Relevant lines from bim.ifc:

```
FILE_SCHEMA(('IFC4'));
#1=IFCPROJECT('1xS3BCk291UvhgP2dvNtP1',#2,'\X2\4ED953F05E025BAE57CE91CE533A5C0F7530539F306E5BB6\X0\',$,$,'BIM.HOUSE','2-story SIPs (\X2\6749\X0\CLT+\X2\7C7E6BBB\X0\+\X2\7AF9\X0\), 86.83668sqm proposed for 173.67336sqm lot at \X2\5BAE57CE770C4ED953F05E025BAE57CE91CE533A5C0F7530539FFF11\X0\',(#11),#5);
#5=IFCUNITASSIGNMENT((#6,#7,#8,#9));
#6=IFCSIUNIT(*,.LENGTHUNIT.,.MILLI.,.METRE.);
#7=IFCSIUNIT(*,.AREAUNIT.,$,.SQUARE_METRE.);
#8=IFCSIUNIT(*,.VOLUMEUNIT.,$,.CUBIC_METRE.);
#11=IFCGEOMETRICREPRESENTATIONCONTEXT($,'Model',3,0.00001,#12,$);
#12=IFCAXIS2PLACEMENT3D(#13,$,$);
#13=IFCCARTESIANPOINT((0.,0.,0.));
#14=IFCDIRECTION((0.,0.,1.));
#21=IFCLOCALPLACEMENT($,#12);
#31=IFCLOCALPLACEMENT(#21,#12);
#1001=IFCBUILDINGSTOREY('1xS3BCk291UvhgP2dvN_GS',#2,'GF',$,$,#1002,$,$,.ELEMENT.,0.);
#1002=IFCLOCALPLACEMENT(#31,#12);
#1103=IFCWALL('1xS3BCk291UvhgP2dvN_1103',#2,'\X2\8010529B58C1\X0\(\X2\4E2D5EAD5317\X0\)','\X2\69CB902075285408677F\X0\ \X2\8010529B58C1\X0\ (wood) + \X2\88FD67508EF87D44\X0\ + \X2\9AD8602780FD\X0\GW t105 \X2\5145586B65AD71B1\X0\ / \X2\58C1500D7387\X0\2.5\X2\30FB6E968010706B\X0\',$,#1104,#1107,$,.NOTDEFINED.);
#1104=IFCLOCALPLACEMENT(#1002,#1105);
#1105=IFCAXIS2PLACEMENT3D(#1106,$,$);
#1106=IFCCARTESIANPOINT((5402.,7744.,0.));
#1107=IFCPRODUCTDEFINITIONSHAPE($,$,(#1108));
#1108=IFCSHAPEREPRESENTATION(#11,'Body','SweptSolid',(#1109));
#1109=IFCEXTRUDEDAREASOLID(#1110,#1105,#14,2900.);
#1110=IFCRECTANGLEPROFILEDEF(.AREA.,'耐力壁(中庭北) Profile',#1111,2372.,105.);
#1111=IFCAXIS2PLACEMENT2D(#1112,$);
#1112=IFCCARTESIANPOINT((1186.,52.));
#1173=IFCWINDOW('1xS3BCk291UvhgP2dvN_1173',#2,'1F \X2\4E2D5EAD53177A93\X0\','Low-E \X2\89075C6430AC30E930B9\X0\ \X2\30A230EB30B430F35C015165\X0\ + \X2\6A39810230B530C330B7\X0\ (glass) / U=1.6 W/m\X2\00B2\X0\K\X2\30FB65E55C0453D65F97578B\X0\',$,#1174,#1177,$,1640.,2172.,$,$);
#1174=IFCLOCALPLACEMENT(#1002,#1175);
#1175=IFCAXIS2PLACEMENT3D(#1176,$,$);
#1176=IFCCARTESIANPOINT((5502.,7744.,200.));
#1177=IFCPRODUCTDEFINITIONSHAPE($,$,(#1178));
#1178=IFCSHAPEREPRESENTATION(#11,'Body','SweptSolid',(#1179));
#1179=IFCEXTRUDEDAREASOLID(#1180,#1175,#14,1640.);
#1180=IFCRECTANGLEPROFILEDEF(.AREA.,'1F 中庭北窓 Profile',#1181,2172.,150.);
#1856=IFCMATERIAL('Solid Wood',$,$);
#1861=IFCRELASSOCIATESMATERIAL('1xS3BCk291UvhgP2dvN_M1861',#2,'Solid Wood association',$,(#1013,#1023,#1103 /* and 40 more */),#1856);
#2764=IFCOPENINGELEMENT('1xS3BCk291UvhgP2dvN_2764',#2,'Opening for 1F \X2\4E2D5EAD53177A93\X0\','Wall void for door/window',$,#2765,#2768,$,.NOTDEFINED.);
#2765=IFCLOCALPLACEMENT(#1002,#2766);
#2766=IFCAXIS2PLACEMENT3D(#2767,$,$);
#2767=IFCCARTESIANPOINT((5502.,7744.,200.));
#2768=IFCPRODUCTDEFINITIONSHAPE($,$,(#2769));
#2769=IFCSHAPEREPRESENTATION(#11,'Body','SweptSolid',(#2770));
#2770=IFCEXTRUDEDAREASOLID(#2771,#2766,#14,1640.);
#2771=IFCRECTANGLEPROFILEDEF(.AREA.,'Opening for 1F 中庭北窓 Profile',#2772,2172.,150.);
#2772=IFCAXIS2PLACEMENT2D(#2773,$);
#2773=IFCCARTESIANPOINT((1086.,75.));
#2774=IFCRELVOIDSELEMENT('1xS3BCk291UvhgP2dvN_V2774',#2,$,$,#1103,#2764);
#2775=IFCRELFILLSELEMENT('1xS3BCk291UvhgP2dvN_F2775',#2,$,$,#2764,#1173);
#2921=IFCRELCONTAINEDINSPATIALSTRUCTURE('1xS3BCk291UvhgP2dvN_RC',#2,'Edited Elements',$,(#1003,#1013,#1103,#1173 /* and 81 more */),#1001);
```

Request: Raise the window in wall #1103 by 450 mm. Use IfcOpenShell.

```python
import numpy as np
import ifcopenshell
import ifcopenshell.api.geometry
import ifcopenshell.util.placement
import ifcopenshell.util.unit

model = ifcopenshell.open("bim.ifc")
unit_scale = ifcopenshell.util.unit.calculate_unit_scale(model)

window = model.by_id(1173)
opening = window.FillsVoids[0].RelatingOpeningElement
dz = 0.45 / unit_scale

shift = np.array([0.0, 0.0, dz])
# The window is not placed relative to its opening, so move both.
for product in (opening, window):
    matrix = ifcopenshell.util.placement.get_local_placement(product.ObjectPlacement)
    matrix[:3, 3] += shift
    ifcopenshell.api.geometry.edit_object_placement(model, product=product, matrix=matrix, is_si=False)

print(f"moved by {dz * unit_scale:+.3f} m")

model.write("bim-out.ifc")
```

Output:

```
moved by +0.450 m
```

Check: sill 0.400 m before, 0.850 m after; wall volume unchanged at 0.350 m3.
